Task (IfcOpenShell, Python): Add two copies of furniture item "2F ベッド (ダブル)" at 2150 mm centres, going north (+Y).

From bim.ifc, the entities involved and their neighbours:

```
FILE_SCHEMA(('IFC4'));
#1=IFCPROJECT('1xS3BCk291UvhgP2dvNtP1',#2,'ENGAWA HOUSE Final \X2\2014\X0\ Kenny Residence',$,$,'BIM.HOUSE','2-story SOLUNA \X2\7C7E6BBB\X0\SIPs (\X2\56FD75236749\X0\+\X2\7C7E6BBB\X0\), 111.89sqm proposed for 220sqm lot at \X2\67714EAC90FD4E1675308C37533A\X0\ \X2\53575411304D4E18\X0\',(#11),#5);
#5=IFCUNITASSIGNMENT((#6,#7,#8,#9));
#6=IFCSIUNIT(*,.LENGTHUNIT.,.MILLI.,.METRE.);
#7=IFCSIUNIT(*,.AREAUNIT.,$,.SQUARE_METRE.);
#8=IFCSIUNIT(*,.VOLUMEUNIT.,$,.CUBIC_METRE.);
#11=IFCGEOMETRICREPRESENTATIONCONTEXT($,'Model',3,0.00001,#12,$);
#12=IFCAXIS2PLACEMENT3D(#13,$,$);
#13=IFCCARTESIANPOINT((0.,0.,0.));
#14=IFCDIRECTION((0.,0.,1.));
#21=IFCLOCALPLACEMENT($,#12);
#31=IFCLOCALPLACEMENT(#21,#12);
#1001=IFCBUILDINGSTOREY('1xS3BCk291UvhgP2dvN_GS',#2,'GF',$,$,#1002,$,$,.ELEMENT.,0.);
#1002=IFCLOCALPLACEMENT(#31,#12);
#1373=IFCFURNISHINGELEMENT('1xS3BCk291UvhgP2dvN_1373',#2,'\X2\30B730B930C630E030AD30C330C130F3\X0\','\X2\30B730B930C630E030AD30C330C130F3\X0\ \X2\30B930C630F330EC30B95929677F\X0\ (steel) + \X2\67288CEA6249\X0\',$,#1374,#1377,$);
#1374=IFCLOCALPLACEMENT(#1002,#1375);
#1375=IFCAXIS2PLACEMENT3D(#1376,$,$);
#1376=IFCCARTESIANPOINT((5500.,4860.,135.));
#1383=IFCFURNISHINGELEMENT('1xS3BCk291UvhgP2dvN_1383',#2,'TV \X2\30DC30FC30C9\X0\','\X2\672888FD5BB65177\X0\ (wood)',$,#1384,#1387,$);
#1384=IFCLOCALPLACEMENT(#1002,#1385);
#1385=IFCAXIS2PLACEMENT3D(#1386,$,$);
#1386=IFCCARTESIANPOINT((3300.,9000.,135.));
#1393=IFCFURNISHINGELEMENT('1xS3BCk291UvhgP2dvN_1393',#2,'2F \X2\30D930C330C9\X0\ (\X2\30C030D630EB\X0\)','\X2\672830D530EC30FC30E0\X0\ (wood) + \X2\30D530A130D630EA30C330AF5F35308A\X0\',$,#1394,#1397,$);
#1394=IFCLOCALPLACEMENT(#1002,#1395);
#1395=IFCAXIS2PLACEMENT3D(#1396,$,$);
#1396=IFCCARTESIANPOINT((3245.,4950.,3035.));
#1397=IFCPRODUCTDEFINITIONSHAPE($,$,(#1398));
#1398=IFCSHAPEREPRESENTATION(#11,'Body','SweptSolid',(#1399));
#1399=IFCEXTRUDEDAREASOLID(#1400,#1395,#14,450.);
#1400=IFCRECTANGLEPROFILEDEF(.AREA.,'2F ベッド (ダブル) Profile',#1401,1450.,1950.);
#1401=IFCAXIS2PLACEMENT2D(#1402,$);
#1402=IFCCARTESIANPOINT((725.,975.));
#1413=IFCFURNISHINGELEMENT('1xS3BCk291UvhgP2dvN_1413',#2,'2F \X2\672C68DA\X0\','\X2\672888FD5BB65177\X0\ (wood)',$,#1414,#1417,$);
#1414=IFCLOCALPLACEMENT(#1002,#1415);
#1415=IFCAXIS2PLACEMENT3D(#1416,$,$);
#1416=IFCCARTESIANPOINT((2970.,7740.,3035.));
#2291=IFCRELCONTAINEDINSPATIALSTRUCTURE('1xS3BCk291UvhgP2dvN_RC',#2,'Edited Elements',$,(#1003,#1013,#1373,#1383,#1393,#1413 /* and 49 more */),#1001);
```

```python
import numpy as np
import ifcopenshell
import ifcopenshell.api.geometry
import ifcopenshell.api.root
import ifcopenshell.util.element
import ifcopenshell.util.placement
import ifcopenshell.util.unit

model = ifcopenshell.open("bim.ifc")
unit_scale = ifcopenshell.util.unit.calculate_unit_scale(model)


def reuse_history(source, copy):
    """copy_class also copies each property set's owner history, people and application; keep the originals."""
    for rel in copy.IsDefinedBy:
        if rel.is_a("IfcRelDefinesByProperties") and (history := rel.RelatingPropertyDefinition.OwnerHistory):
            rel.RelatingPropertyDefinition.OwnerHistory = source.OwnerHistory
            ifcopenshell.util.element.remove_deep2(model, history)


source = model.by_guid("1xS3BCk291UvhgP2dvN_1393")
base = ifcopenshell.util.placement.get_local_placement(source.ObjectPlacement)
step = np.array([0.0, 1.0, 0.0]) * 2.15 / unit_scale

for i in range(1, 3):
    copy = ifcopenshell.api.root.copy_class(model, product=source)
    copy.Representation = ifcopenshell.util.element.copy_deep(
        model, source.Representation, exclude=["IfcGeometricRepresentationContext", "IfcRepresentationMap"]
    )
    reuse_history(source, copy)
    matrix = base.copy()
    matrix[:3, 3] += i * step
    print("added at", matrix[:3, 3].round(3) + 0.0)
    ifcopenshell.api.geometry.edit_object_placement(model, product=copy, matrix=matrix, is_si=False)

model.write("bim_rev.ifc")
```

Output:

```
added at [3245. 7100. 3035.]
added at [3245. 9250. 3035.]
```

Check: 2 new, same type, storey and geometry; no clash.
